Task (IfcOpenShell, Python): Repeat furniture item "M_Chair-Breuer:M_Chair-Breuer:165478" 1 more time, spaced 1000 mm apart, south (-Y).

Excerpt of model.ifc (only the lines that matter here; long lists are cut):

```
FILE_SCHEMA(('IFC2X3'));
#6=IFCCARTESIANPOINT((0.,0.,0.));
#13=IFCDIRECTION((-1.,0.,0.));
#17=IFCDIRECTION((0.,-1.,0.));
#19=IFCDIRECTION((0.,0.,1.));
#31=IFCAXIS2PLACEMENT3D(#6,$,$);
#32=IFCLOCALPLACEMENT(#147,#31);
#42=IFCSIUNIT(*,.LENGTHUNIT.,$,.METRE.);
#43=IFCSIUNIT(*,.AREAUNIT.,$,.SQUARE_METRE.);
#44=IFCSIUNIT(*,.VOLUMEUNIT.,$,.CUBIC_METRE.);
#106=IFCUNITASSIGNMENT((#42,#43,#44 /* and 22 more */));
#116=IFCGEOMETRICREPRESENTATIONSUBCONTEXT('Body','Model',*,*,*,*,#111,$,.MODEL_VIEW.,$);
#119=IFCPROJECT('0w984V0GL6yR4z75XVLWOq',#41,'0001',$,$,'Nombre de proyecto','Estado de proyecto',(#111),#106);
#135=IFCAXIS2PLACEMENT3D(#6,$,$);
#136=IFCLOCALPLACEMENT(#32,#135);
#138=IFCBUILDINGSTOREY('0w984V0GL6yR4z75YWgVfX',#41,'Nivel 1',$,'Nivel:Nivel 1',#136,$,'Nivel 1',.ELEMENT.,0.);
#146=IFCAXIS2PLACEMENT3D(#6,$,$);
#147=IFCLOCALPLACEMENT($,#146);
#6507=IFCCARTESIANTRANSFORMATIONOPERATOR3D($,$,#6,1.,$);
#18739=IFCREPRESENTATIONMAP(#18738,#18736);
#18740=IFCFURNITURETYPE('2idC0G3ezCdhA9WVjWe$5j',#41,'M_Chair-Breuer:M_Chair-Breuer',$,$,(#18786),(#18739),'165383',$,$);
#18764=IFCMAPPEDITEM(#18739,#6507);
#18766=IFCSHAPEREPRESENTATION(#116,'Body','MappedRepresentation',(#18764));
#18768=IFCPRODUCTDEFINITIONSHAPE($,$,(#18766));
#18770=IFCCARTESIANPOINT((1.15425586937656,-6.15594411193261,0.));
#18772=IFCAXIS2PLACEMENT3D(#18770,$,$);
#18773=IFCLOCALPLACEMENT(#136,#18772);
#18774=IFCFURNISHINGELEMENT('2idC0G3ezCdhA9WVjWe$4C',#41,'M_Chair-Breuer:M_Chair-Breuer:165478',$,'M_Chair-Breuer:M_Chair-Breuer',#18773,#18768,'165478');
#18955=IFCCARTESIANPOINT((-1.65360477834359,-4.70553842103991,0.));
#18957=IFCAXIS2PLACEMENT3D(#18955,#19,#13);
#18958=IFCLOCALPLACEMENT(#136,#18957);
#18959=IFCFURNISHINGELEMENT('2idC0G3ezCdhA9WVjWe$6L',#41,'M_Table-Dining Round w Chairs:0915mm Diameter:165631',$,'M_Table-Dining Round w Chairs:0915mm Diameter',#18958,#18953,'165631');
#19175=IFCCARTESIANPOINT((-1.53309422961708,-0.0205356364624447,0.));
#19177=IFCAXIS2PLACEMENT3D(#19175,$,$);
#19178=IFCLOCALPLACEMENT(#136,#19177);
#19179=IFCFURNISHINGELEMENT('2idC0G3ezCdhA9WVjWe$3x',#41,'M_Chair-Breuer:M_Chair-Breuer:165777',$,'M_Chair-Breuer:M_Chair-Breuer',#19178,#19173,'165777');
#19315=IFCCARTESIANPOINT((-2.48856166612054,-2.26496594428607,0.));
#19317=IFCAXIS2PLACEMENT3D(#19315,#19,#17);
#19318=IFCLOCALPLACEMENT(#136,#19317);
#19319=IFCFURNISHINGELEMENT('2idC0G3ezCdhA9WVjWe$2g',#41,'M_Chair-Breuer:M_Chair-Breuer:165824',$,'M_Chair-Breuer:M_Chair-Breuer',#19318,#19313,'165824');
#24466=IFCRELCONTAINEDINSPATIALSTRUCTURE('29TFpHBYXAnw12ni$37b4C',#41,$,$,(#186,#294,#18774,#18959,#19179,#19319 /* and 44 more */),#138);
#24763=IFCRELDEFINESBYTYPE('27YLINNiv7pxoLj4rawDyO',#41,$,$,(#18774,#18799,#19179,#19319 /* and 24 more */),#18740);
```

```python
import numpy as np
import ifcopenshell
import ifcopenshell.api.geometry
import ifcopenshell.api.root
import ifcopenshell.util.element
import ifcopenshell.util.placement
import ifcopenshell.util.unit

model = ifcopenshell.open("model.ifc")
unit_scale = ifcopenshell.util.unit.calculate_unit_scale(model)


def reuse_history(source, copy):
    """copy_class also copies each property set's owner history, people and application; keep the originals."""
    for rel in copy.IsDefinedBy:
        if rel.is_a("IfcRelDefinesByProperties") and (history := rel.RelatingPropertyDefinition.OwnerHistory):
            rel.RelatingPropertyDefinition.OwnerHistory = source.OwnerHistory
            ifcopenshell.util.element.remove_deep2(model, history)


source = model.by_id(18774)
base = ifcopenshell.util.placement.get_local_placement(source.ObjectPlacement)
step = np.array([0.0, -1.0, 0.0]) * 1 / unit_scale

for i in range(1, 2):
    copy = ifcopenshell.api.root.copy_class(model, product=source)
    copy.Representation = ifcopenshell.util.element.copy_deep(
        model, source.Representation, exclude=["IfcGeometricRepresentationContext", "IfcRepresentationMap"]
    )
    copy.Name = "M_Chair-Breuer:M_Chair-Breuer"
    copy.Tag = None
    reuse_history(source, copy)
    matrix = base.copy()
    matrix[:3, 3] += i * step
    print("added at", matrix[:3, 3].round(3) + 0.0)
    ifcopenshell.api.geometry.edit_object_placement(model, product=copy, matrix=matrix, is_si=False)

model.write("model_updated.ifc")
```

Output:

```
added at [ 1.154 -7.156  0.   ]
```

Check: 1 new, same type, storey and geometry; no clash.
